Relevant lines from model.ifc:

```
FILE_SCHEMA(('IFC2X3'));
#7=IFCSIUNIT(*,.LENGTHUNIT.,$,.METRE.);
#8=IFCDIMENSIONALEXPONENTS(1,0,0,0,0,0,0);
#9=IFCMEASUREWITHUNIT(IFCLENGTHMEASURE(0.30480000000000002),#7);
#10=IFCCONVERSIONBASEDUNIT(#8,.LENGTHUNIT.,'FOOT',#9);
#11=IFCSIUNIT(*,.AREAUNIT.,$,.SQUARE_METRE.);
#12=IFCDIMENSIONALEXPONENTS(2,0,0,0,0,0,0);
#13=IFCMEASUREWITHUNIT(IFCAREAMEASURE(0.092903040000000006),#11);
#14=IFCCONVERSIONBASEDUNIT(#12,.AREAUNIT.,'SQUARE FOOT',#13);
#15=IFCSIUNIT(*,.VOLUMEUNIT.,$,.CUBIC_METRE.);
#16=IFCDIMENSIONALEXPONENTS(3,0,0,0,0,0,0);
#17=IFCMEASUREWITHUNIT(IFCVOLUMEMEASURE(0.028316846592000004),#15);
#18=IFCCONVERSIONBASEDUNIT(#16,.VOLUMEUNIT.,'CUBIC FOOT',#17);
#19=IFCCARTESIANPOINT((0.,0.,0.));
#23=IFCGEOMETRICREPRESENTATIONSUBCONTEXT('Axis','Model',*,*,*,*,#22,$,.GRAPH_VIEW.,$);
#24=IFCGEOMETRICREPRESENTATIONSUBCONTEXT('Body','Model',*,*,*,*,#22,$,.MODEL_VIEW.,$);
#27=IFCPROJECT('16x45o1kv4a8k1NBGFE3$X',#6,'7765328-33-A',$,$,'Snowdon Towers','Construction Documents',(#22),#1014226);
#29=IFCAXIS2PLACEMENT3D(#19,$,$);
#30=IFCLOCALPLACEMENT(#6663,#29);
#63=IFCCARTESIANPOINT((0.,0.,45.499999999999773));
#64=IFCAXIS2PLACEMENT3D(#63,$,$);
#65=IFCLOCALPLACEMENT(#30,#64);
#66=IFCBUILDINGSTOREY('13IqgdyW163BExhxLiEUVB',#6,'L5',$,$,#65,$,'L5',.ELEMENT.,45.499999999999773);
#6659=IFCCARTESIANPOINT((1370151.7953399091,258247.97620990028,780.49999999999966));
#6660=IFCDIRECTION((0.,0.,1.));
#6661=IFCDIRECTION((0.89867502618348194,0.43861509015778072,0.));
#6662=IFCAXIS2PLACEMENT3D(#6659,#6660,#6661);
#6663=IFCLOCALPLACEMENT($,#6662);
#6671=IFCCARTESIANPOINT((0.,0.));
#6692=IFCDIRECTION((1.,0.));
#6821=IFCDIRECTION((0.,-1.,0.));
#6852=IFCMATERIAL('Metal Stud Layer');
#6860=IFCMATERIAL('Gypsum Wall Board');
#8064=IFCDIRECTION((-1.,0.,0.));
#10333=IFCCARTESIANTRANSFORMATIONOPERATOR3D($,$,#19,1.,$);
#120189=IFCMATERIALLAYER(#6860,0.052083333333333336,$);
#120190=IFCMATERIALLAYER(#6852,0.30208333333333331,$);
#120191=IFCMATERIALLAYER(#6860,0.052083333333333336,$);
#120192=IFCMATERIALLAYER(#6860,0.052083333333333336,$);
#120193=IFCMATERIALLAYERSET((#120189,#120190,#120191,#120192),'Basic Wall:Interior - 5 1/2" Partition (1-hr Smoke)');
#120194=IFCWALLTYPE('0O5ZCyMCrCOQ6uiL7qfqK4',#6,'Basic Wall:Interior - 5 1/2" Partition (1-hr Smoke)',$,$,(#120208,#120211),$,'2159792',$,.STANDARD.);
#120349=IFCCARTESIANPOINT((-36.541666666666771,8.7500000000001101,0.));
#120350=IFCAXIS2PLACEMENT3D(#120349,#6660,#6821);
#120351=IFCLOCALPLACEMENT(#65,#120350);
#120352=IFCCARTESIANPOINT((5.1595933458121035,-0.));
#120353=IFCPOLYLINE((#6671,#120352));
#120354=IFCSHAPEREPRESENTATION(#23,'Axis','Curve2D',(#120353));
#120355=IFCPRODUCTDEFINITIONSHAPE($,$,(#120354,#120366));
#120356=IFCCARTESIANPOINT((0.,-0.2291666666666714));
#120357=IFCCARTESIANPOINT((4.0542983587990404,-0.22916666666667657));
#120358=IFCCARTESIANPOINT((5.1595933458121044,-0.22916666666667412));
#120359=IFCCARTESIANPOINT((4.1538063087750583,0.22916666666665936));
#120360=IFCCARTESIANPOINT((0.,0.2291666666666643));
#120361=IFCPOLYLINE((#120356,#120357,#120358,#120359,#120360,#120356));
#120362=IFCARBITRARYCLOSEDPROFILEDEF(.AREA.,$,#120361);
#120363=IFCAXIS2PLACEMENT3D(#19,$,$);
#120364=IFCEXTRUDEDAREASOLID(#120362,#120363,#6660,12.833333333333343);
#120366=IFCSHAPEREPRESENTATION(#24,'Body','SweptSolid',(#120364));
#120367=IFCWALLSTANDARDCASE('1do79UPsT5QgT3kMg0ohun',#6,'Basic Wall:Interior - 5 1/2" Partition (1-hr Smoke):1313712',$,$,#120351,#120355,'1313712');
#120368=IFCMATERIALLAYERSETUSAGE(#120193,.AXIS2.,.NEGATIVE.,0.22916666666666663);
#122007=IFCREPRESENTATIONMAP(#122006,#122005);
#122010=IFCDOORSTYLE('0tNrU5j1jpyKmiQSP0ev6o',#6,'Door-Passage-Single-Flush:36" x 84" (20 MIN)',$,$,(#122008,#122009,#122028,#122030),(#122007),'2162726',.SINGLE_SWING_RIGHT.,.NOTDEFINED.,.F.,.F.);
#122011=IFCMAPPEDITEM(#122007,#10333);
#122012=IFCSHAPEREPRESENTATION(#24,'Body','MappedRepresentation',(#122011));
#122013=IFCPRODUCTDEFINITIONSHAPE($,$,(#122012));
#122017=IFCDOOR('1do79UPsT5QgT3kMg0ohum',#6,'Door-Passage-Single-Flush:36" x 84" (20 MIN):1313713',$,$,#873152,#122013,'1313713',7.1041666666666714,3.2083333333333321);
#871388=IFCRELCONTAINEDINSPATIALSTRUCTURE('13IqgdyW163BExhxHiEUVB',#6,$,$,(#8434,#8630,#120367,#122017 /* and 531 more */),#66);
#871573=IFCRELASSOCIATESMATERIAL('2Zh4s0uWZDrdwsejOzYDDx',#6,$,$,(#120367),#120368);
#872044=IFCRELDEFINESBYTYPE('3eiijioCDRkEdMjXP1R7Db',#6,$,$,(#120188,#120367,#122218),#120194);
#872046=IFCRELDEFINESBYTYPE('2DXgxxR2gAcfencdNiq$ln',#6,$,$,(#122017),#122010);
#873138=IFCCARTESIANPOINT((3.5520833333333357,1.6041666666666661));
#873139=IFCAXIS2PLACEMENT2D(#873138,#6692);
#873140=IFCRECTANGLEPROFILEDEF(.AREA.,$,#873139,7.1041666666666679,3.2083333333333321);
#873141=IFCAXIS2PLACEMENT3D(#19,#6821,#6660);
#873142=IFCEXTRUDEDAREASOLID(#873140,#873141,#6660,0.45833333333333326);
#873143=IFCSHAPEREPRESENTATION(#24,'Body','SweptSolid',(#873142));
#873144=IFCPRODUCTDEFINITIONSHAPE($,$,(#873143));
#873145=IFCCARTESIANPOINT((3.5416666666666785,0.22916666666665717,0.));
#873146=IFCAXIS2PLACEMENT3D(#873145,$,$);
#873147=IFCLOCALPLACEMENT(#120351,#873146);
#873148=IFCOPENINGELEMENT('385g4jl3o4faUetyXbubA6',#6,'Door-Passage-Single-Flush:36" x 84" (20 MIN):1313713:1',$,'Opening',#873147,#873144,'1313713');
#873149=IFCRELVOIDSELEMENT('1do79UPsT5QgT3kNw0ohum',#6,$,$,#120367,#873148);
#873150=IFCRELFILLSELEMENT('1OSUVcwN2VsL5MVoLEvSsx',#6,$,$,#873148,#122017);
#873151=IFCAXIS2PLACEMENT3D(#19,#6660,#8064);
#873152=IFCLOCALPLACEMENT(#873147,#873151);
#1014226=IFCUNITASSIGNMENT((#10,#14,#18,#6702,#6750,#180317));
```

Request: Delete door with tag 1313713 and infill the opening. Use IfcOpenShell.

```python
import ifcopenshell
import ifcopenshell.api.feature
import ifcopenshell.api.root
import ifcopenshell.geom
import ifcopenshell.util.shape

model = ifcopenshell.open("model.ifc")
settings = ifcopenshell.geom.settings()


def volume(element):
    """Net volume in cubic metres, openings subtracted."""
    shape = ifcopenshell.geom.create_shape(settings, element)
    return ifcopenshell.util.shape.get_volume(shape.geometry)


door = model.by_guid("1do79UPsT5QgT3kMg0ohum")
opening = door.FillsVoids[0].RelatingOpeningElement
wall = opening.VoidsElements[0].RelatingBuildingElement
before = volume(wall)

ifcopenshell.api.root.remove_product(model, product=door)
ifcopenshell.api.feature.remove_feature(model, feature=opening)

after = volume(wall)

print(f"wall volume {before:.3f} -> {after:.3f} m3")

model.write("model_updated.ifc")
```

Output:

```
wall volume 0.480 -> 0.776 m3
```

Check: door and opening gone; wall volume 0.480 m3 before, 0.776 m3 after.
